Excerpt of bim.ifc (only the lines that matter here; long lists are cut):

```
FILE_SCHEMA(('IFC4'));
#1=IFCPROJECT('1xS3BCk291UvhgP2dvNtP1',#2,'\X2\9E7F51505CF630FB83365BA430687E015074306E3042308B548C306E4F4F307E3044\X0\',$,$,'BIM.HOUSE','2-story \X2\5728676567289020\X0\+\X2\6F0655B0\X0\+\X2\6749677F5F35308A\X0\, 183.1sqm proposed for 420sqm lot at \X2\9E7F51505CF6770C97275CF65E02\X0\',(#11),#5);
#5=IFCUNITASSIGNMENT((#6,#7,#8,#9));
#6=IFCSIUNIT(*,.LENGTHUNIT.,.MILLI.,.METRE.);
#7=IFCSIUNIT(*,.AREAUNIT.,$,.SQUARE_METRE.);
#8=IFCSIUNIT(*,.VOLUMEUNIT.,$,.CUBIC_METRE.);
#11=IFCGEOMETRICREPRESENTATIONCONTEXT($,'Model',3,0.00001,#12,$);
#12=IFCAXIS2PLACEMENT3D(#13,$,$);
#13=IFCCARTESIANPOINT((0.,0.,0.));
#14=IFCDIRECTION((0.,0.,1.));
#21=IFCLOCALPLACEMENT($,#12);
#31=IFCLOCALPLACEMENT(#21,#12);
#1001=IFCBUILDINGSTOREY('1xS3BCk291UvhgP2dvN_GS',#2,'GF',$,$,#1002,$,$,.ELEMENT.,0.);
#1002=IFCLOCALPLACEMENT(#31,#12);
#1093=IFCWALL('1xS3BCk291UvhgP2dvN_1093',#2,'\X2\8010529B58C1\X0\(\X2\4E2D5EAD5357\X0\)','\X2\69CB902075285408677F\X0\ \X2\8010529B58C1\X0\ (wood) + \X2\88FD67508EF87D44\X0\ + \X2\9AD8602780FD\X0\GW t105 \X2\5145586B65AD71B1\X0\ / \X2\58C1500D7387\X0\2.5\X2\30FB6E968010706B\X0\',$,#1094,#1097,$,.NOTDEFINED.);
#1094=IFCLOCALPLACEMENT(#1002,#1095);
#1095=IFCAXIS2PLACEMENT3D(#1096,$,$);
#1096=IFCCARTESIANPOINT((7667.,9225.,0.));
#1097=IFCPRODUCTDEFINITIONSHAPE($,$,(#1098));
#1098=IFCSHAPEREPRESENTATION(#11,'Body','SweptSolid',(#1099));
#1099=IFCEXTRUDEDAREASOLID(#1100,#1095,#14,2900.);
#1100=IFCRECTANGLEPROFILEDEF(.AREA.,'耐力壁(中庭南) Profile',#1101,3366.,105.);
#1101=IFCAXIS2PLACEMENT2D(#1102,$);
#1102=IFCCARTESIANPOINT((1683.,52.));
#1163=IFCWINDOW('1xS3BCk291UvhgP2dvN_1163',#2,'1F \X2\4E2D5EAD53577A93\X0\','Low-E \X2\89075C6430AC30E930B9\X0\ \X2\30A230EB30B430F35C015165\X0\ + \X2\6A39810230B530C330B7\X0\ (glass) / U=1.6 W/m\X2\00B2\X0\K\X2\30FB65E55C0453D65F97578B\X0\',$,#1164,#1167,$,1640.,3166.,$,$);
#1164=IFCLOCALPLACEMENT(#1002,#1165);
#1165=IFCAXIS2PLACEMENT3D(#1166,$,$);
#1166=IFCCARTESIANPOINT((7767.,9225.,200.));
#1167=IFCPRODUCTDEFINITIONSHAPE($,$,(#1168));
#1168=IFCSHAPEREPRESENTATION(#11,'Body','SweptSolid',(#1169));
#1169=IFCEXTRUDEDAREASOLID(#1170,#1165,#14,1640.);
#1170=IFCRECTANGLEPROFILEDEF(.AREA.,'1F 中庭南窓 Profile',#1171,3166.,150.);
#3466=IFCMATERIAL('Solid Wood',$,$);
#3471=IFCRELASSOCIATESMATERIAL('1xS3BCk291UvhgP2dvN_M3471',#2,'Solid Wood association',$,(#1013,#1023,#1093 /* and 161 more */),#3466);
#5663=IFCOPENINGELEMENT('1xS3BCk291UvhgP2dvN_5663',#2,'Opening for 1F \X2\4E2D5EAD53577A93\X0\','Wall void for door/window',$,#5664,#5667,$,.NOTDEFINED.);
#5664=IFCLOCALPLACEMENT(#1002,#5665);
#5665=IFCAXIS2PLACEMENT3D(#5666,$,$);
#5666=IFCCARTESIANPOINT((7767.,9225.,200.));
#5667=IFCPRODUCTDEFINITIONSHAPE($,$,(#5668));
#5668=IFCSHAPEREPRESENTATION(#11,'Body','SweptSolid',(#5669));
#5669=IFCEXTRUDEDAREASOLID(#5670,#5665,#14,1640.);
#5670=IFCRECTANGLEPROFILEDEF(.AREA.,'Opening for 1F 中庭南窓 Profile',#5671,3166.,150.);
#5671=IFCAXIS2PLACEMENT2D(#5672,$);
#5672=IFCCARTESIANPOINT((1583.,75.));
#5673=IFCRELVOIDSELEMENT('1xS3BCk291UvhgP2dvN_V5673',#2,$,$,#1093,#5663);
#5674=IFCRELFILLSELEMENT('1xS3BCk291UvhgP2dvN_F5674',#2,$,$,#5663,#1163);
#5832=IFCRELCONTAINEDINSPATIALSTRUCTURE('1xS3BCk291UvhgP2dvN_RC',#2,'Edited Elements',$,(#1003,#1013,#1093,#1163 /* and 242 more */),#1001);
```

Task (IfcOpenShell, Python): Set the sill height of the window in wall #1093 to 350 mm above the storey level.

```python
import numpy as np
import ifcopenshell
import ifcopenshell.api.geometry
import ifcopenshell.geom
import ifcopenshell.util.element
import ifcopenshell.util.placement
import ifcopenshell.util.shape
import ifcopenshell.util.unit

model = ifcopenshell.open("bim.ifc")
unit_scale = ifcopenshell.util.unit.calculate_unit_scale(model)

window = model.by_guid("1xS3BCk291UvhgP2dvN_1163")
opening = window.FillsVoids[0].RelatingOpeningElement
storey = ifcopenshell.util.element.get_container(window, ifc_class="IfcBuildingStorey")
level = ifcopenshell.util.placement.get_local_placement(storey.ObjectPlacement)[2, 3]

# The opening's origin need not be at the sill, so measure its lowest point.
shape = ifcopenshell.geom.create_shape(ifcopenshell.geom.settings(), opening)
bottom = ifcopenshell.util.shape.get_shape_bottom_elevation(shape, shape.geometry) / unit_scale
dz = level + 350.0 - bottom

shift = np.array([0.0, 0.0, dz])
# The window is not placed relative to its opening, so move both.
for product in (opening, window):
    matrix = ifcopenshell.util.placement.get_local_placement(product.ObjectPlacement)
    matrix[:3, 3] += shift
    ifcopenshell.api.geometry.edit_object_placement(model, product=product, matrix=matrix, is_si=False)

print(f"moved by {dz * unit_scale:+.3f} m")

model.write("bim_v2.ifc")
```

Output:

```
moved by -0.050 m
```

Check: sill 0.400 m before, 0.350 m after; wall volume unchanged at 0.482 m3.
